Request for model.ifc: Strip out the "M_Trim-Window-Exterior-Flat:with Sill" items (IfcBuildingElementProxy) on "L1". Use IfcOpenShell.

First a look at what the model holds.

```python
import ifcopenshell
import ifcopenshell.util.element

model = ifcopenshell.open("model.ifc")
print(model.schema)
storey = next(s for s in model.by_type("IfcBuildingStorey") if s.Name == "L1")
proxies = [e for e in ifcopenshell.util.element.get_decomposition(storey) if e.is_a("IfcBuildingElementProxy")]
seen = {}
for e in proxies:
    element_type = ifcopenshell.util.element.get_type(e)
    name = element_type.Name if element_type not in (None, e) else None
    seen[name] = seen.get(name, 0) + 1
for name, count in sorted(seen.items(), key=str):
    print(count, "x", name)
```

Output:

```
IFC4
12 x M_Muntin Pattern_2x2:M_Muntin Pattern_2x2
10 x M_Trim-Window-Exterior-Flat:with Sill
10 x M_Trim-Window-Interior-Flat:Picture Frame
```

```python
import ifcopenshell
import ifcopenshell.api.root
import ifcopenshell.util.element

model = ifcopenshell.open("model.ifc")

storey = next(s for s in model.by_type("IfcBuildingStorey") if s.Name == "L1")
proxies = [e for e in ifcopenshell.util.element.get_decomposition(storey) if e.is_a("IfcBuildingElementProxy")]
targets = [e for e in proxies if (t := ifcopenshell.util.element.get_type(e)) not in (None, e) and t.Name == "M_Trim-Window-Exterior-Flat:with Sill"]

for e in targets:
    ifcopenshell.api.root.remove_product(model, product=e)
print(len(targets), "removed")

model.write("model_updated.ifc")
```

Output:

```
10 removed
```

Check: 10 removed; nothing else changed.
